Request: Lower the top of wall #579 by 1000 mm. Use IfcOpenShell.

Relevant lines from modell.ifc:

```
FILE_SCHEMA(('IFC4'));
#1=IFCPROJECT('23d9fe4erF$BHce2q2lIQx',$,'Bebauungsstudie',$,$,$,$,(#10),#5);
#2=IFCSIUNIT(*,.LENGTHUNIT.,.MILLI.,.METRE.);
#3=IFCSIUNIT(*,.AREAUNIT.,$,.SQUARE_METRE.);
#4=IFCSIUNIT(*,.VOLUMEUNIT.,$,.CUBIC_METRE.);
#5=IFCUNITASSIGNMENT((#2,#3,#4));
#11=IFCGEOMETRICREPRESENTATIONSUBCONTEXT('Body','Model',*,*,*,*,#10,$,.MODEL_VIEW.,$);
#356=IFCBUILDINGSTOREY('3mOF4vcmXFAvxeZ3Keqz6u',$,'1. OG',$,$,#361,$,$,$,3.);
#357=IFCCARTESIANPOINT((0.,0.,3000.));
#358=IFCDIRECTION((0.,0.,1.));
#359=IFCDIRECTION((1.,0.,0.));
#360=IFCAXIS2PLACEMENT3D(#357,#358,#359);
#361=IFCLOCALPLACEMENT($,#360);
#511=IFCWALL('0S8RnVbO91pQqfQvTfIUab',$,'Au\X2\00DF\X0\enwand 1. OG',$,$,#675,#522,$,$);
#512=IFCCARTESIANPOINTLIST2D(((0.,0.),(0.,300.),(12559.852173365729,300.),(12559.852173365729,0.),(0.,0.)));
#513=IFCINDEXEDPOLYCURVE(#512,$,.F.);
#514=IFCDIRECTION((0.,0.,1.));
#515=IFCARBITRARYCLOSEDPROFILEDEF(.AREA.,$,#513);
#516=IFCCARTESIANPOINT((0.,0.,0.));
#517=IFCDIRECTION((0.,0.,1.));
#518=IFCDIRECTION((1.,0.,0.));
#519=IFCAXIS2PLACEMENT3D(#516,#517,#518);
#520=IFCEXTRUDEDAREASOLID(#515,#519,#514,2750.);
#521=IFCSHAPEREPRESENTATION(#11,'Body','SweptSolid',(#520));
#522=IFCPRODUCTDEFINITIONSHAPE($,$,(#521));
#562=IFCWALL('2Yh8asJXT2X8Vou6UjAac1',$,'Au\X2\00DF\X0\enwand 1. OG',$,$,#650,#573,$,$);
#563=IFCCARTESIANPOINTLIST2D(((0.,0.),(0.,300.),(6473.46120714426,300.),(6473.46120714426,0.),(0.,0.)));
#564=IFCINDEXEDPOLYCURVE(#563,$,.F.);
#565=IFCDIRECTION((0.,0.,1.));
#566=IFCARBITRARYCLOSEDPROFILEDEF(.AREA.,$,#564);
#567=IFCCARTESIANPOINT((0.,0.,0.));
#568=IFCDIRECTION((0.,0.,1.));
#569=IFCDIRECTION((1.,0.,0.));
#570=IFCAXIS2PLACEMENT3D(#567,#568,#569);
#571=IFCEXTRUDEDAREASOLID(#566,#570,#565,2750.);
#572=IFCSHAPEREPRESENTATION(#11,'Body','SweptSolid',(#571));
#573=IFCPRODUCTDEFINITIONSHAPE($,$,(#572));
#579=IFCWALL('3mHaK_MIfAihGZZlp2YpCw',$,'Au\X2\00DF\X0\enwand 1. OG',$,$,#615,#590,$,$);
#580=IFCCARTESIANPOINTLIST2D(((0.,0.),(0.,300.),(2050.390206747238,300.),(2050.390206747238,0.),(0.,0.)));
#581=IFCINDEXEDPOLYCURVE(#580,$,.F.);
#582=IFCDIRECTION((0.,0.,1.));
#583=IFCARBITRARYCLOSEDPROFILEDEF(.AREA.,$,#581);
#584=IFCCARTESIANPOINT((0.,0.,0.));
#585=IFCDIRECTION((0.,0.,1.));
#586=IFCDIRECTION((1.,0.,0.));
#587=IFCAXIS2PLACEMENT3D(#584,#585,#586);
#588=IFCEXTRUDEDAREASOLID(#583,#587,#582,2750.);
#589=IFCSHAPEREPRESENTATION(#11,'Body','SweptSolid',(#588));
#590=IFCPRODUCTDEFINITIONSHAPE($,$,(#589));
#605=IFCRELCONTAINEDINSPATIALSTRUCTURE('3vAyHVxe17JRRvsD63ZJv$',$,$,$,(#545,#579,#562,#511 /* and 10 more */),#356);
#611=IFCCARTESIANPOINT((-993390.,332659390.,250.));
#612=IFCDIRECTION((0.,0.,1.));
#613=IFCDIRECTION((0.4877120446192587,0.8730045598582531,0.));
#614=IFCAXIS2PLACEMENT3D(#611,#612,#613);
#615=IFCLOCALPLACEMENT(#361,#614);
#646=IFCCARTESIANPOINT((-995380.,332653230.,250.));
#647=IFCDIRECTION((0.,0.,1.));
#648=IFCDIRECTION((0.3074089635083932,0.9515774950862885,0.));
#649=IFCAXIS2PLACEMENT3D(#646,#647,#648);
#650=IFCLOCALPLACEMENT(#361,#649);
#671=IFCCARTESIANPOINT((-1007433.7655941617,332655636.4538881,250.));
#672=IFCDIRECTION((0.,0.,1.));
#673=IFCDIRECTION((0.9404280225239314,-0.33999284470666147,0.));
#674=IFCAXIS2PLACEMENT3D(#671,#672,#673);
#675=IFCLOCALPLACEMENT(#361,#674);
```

```python
import ifcopenshell
import ifcopenshell.geom
import ifcopenshell.util.representation
import ifcopenshell.util.shape

model = ifcopenshell.open("modell.ifc")
settings = ifcopenshell.geom.settings()


def volume(element):
    """Net volume in cubic metres, openings subtracted."""
    shape = ifcopenshell.geom.create_shape(settings, element)
    return ifcopenshell.util.shape.get_volume(shape.geometry)


wall = model.by_id(579)
before = volume(wall)

body = ifcopenshell.util.representation.get_representation(wall, "Model", "Body")
solid = body.Items[0]
old_height = solid.Depth
solid.Depth -= 1000.0
after = volume(wall)

print(f"height {old_height:g} -> {solid.Depth:g}, volume {before:.3f} -> {after:.3f} m3")

model.write("modell_v2.ifc")
```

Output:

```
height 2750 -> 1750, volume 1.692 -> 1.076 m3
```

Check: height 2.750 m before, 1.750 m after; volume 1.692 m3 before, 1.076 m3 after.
